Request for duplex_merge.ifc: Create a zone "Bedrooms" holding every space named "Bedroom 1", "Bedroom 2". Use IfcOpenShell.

First a look at what the model holds.

```python
import ifcopenshell

model = ifcopenshell.open("duplex_merge.ifc")
print(model.schema)
seen = {}
for space in model.by_type("IfcSpace"):
    seen[space.LongName] = seen.get(space.LongName, 0) + 1
for name, count in sorted(seen.items(), key=str):
    print(count, "x", name)
print("zones:", [z.Name for z in model.by_type("IfcZone")][:20])
```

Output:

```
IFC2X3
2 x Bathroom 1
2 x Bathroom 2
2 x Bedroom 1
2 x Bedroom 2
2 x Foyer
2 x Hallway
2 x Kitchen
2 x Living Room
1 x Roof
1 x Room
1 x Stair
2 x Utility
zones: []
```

```python
import ifcopenshell
import ifcopenshell.api.group
import ifcopenshell.api.root

model = ifcopenshell.open("duplex_merge.ifc")

names = {"Bedroom 1", "Bedroom 2"}
spaces = [s for s in model.by_type("IfcSpace") if s.LongName in names]

zone = ifcopenshell.api.root.create_entity(model, ifc_class="IfcZone", name="Bedrooms")
ifcopenshell.api.group.assign_group(model, products=spaces, group=zone)
print(len(spaces), "spaces in", zone.Name)

model.write("duplex_merge-out.ifc")
```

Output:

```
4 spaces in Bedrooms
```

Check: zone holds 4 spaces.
